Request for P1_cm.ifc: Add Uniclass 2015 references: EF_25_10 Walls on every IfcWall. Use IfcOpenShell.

First a look at what the model holds.

```python
import ifcopenshell

model = ifcopenshell.open("P1_cm.ifc")
print(model.schema)
print("classifications:", [c.Name for c in model.by_type("IfcClassification")])
for ifc_class in ("IfcDoor", "IfcRoof", "IfcStair", "IfcWall", "IfcWindow"):
    print(ifc_class, len(model.by_type(ifc_class)))
```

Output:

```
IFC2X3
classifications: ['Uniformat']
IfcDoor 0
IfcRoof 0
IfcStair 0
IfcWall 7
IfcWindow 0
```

```python
import ifcopenshell
import ifcopenshell.api.classification

model = ifcopenshell.open("P1_cm.ifc")

# IFC2X3 requires Source and Edition and has no link from the project to the system.
system = model.create_entity("IfcClassification", Source="NBS", Edition="2015", Name="Uniclass 2015")

codes = {
    "IfcWall": ("EF_25_10", "Walls"),
}
for ifc_class, (code, name) in codes.items():
    products = model.by_type(ifc_class)
    ifcopenshell.api.classification.add_reference(
        model, products=products, classification=system, identification=code, name=name
    )
    print(code, len(products))

model.write("P1_cm_updated.ifc")
```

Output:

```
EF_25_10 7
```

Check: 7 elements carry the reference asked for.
